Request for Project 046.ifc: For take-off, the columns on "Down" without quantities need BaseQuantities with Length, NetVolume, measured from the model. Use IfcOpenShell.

First a look at what the model holds.

```python
import ifcopenshell
import ifcopenshell.util.element
import ifcopenshell.util.unit

model = ifcopenshell.open("Project 046.ifc")
print(model.schema)
for unit_type in ("LENGTHUNIT", "AREAUNIT", "VOLUMEUNIT"):
    print(unit_type, ifcopenshell.util.unit.calculate_unit_scale(model, unit_type))
storey = next(s for s in model.by_type("IfcBuildingStorey") if s.Name == "Down")
columns = [e for e in ifcopenshell.util.element.get_decomposition(storey) if e.is_a("IfcColumn")]
for e in sorted(columns, key=lambda e: e.id()):
    print(e.id(), e.is_a(), e.Name, list(ifcopenshell.util.element.get_psets(e, qtos_only=True)), sep=" | ")
```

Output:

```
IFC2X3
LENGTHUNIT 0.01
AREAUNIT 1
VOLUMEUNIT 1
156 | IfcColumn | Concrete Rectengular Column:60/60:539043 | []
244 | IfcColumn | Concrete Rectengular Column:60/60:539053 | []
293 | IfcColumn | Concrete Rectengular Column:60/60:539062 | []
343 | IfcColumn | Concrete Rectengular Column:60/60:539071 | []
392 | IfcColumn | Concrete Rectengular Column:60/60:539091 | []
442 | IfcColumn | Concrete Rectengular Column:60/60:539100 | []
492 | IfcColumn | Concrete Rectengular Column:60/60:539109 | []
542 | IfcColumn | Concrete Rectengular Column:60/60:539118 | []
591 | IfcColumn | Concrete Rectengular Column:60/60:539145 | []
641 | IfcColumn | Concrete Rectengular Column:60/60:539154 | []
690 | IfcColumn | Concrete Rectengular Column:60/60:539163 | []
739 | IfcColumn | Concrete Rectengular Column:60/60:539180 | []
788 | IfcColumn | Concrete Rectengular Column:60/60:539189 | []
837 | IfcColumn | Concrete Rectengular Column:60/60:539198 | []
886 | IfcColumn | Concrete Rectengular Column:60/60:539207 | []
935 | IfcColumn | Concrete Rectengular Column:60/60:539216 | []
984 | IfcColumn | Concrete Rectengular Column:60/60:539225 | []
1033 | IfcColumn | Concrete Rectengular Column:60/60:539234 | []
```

```python
import ifcopenshell
import ifcopenshell.api.pset
import ifcopenshell.geom
import ifcopenshell.util.element
import ifcopenshell.util.shape
import ifcopenshell.util.unit

model = ifcopenshell.open("Project 046.ifc")
unit_scale = ifcopenshell.util.unit.calculate_unit_scale(model)
volume_scale = ifcopenshell.util.unit.calculate_unit_scale(model, "VOLUMEUNIT")
settings = ifcopenshell.geom.settings()

storey = next(s for s in model.by_type("IfcBuildingStorey") if s.Name == "Down")
columns = [e for e in ifcopenshell.util.element.get_decomposition(storey) if e.is_a("IfcColumn")]

for e in sorted(columns, key=lambda e: e.id()):
    if ifcopenshell.util.element.get_psets(e, qtos_only=True, should_inherit=False):
        continue
    # Geometry comes back in metres, in the element's own axes.
    shape = ifcopenshell.geom.create_shape(settings, e)
    values = {
        "Length": ifcopenshell.util.shape.get_z(shape.geometry) / unit_scale,
        "NetVolume": ifcopenshell.util.shape.get_volume(shape.geometry) / volume_scale,
    }
    qto = ifcopenshell.api.pset.add_qto(model, product=e, name="BaseQuantities")
    ifcopenshell.api.pset.edit_qto(model, qto=qto, properties=values)
    print(e.id(), {k: round(v, 3) for k, v in values.items()})

model.write("Project 046_v2.ifc")
```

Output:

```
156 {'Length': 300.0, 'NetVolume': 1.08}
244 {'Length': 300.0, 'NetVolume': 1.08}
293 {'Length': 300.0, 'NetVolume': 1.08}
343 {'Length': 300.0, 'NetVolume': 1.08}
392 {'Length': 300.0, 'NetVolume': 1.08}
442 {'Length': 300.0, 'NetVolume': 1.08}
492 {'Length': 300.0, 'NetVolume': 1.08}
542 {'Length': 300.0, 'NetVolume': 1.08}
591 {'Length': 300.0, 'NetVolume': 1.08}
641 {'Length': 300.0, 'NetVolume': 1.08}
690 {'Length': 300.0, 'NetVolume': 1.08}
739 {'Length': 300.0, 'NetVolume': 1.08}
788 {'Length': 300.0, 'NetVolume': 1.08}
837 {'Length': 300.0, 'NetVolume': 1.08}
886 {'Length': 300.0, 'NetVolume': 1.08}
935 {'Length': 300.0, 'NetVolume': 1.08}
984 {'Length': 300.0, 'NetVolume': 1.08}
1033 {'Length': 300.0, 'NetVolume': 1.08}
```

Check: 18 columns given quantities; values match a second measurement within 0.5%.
